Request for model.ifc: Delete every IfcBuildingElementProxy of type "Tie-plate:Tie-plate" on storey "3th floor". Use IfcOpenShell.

First a look at what the model holds.

```python
import ifcopenshell
import ifcopenshell.util.element

model = ifcopenshell.open("model.ifc")
print(model.schema)
storey = next(s for s in model.by_type("IfcBuildingStorey") if s.Name == "3th floor")
proxies = [e for e in ifcopenshell.util.element.get_decomposition(storey) if e.is_a("IfcBuildingElementProxy")]
seen = {}
for e in proxies:
    element_type = ifcopenshell.util.element.get_type(e)
    name = element_type.Name if element_type not in (None, e) else None
    seen[name] = seen.get(name, 0) + 1
for name, count in sorted(seen.items(), key=str):
    print(count, "x", name)
```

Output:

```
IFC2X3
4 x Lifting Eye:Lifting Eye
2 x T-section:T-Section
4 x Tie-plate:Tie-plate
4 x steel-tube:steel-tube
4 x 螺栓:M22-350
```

```python
import ifcopenshell
import ifcopenshell.api.root
import ifcopenshell.util.element

model = ifcopenshell.open("model.ifc")

storey = next(s for s in model.by_type("IfcBuildingStorey") if s.Name == "3th floor")
proxies = [e for e in ifcopenshell.util.element.get_decomposition(storey) if e.is_a("IfcBuildingElementProxy")]
targets = [e for e in proxies if (t := ifcopenshell.util.element.get_type(e)) not in (None, e) and t.Name == "Tie-plate:Tie-plate"]

for e in targets:
    ifcopenshell.api.root.remove_product(model, product=e)
print(len(targets), "removed")

model.write("model_updated.ifc")
```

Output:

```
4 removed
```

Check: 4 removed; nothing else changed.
